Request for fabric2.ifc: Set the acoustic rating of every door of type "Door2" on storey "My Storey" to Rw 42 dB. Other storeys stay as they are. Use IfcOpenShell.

First a look at what the model holds.

```python
import ifcopenshell
import ifcopenshell.util.element

model = ifcopenshell.open("fabric2.ifc")
print(model.schema)
storey = next(s for s in model.by_type("IfcBuildingStorey") if s.Name == "My Storey")
doors = [e for e in ifcopenshell.util.element.get_decomposition(storey) if e.is_a("IfcDoor")]
seen = {}
for e in doors:
    element_type = ifcopenshell.util.element.get_type(e)
    key = (element_type.Name if element_type != e and element_type else None, ifcopenshell.util.element.get_pset(e, "Pset_DoorCommon", "AcousticRating"))
    seen[key] = seen.get(key, 0) + 1
for (name, value), count in sorted(seen.items(), key=str):
    print(count, "x", name, "|", value)
```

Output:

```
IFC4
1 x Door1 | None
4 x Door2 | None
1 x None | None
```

```python
import ifcopenshell
import ifcopenshell.api.pset
import ifcopenshell.util.element

model = ifcopenshell.open("fabric2.ifc")

storey = next(s for s in model.by_type("IfcBuildingStorey") if s.Name == "My Storey")
doors = [e for e in ifcopenshell.util.element.get_decomposition(storey) if e.is_a("IfcDoor")]

count = 0
for e in doors:
    element_type = ifcopenshell.util.element.get_type(e)
    if element_type in (None, e) or element_type.Name != "Door2":
        continue
    # add_pset returns the element's existing set when there is one.
    pset = ifcopenshell.api.pset.add_pset(model, product=e, name="Pset_DoorCommon")
    ifcopenshell.api.pset.edit_pset(model, pset=pset, properties={"AcousticRating": "Rw 42 dB"})
    count += 1

print(count, "doors updated")

model.write("fabric2_updated.ifc")
```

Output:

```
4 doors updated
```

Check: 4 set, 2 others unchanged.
